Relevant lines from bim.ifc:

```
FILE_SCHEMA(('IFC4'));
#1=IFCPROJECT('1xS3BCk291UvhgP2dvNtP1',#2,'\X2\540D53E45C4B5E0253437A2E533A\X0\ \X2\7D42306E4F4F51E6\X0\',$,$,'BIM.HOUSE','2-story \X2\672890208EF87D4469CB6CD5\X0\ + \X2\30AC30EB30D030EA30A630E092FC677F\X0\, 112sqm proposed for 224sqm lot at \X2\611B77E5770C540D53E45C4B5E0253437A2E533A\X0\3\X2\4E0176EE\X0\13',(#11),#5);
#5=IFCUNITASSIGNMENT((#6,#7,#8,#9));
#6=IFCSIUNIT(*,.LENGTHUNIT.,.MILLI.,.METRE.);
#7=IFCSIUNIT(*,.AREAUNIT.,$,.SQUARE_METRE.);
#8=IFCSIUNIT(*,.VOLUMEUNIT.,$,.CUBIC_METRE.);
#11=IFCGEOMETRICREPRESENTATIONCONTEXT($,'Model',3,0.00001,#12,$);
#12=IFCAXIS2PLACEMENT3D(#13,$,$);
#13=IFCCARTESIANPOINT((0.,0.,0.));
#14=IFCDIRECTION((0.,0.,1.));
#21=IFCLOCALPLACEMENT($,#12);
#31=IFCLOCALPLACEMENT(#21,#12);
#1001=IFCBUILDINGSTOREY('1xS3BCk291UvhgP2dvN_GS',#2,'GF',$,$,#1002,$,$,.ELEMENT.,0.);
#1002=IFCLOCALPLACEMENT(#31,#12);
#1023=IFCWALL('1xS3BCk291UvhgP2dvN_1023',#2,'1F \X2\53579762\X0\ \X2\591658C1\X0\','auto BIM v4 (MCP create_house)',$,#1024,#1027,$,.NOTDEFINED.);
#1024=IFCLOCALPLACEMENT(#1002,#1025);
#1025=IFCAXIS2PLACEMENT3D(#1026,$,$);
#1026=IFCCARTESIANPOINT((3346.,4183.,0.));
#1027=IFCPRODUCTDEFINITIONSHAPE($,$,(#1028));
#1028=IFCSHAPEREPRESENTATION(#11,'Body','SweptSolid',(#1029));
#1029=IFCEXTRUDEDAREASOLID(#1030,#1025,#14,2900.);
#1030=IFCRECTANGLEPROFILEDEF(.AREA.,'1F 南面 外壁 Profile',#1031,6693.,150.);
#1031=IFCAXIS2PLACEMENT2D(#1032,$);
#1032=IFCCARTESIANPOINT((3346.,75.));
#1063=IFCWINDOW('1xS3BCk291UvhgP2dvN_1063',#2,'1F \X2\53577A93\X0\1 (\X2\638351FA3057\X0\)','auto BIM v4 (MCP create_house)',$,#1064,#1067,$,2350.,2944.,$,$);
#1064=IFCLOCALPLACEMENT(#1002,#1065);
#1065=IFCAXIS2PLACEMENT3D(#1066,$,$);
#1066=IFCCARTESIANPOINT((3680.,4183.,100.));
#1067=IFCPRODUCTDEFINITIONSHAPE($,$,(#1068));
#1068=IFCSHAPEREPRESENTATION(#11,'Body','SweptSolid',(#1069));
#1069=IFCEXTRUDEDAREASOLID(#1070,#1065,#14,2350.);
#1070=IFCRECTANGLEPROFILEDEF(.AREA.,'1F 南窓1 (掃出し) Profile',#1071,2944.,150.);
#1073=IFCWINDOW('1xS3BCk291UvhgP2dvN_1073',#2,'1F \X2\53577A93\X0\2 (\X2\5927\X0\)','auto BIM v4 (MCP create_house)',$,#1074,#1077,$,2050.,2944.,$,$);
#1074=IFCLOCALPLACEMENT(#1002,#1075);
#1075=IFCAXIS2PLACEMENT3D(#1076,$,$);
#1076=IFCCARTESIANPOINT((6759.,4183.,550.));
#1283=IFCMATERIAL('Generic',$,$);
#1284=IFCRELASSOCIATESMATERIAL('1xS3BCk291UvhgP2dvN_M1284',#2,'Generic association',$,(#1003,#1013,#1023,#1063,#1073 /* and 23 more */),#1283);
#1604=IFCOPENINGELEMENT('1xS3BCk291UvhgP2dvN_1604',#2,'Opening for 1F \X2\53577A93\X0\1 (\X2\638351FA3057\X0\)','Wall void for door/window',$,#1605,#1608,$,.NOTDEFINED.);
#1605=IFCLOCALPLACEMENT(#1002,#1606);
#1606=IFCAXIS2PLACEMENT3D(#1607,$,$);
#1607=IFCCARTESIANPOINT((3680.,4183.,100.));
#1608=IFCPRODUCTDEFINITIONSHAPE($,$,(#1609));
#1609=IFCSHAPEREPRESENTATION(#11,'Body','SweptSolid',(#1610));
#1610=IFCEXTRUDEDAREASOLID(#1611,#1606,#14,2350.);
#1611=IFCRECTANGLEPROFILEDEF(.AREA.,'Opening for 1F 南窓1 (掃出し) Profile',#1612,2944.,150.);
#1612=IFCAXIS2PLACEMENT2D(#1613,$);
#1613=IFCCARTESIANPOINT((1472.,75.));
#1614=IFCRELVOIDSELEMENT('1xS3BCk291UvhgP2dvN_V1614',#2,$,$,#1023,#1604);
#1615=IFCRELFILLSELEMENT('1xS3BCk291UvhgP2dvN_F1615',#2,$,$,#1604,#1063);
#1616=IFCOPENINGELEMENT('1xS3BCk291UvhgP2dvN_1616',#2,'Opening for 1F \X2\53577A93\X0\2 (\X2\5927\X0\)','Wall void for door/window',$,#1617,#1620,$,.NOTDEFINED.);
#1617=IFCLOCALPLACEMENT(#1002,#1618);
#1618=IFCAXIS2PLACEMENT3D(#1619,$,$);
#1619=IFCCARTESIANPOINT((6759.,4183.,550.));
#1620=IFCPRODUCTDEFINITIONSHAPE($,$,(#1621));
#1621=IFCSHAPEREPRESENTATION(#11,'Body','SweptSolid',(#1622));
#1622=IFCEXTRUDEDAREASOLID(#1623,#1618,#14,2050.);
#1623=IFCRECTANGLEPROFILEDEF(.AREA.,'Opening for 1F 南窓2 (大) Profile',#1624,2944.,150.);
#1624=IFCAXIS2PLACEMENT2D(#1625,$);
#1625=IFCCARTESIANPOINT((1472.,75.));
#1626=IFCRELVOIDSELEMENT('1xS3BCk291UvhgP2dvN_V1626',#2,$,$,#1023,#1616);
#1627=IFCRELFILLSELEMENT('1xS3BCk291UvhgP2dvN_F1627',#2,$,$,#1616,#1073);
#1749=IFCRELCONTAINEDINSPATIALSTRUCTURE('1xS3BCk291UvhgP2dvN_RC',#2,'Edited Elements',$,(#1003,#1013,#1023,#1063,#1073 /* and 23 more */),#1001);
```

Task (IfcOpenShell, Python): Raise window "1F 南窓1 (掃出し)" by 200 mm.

```python
import numpy as np
import ifcopenshell
import ifcopenshell.api.geometry
import ifcopenshell.util.placement
import ifcopenshell.util.unit

model = ifcopenshell.open("bim.ifc")
unit_scale = ifcopenshell.util.unit.calculate_unit_scale(model)

window = model.by_guid("1xS3BCk291UvhgP2dvN_1063")
opening = window.FillsVoids[0].RelatingOpeningElement
dz = 0.2 / unit_scale

shift = np.array([0.0, 0.0, dz])
# The window is not placed relative to its opening, so move both.
for product in (opening, window):
    matrix = ifcopenshell.util.placement.get_local_placement(product.ObjectPlacement)
    matrix[:3, 3] += shift
    ifcopenshell.api.geometry.edit_object_placement(model, product=product, matrix=matrix, is_si=False)

print(f"moved by {dz * unit_scale:+.3f} m")

model.write("bim-out.ifc")
```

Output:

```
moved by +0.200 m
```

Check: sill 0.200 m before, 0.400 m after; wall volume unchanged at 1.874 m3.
